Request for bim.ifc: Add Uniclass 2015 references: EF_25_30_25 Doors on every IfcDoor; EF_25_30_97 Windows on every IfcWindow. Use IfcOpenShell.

First a look at what the model holds.

```python
import ifcopenshell

model = ifcopenshell.open("bim.ifc")
print(model.schema)
print("classifications:", [c.Name for c in model.by_type("IfcClassification")])
for ifc_class in ("IfcDoor", "IfcRoof", "IfcStair", "IfcWall", "IfcWindow"):
    print(ifc_class, len(model.by_type(ifc_class)))
```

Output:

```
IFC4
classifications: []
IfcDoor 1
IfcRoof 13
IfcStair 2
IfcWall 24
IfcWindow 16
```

```python
import ifcopenshell
import ifcopenshell.api.classification

model = ifcopenshell.open("bim.ifc")

system = ifcopenshell.api.classification.add_classification(model, classification="Uniclass 2015")

codes = {
    "IfcDoor": ("EF_25_30_25", "Doors"),
    "IfcWindow": ("EF_25_30_97", "Windows"),
}
for ifc_class, (code, name) in codes.items():
    products = model.by_type(ifc_class)
    ifcopenshell.api.classification.add_reference(
        model, products=products, classification=system, identification=code, name=name
    )
    print(code, len(products))

model.write("bim_updated.ifc")
```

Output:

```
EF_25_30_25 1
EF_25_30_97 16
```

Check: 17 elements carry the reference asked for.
